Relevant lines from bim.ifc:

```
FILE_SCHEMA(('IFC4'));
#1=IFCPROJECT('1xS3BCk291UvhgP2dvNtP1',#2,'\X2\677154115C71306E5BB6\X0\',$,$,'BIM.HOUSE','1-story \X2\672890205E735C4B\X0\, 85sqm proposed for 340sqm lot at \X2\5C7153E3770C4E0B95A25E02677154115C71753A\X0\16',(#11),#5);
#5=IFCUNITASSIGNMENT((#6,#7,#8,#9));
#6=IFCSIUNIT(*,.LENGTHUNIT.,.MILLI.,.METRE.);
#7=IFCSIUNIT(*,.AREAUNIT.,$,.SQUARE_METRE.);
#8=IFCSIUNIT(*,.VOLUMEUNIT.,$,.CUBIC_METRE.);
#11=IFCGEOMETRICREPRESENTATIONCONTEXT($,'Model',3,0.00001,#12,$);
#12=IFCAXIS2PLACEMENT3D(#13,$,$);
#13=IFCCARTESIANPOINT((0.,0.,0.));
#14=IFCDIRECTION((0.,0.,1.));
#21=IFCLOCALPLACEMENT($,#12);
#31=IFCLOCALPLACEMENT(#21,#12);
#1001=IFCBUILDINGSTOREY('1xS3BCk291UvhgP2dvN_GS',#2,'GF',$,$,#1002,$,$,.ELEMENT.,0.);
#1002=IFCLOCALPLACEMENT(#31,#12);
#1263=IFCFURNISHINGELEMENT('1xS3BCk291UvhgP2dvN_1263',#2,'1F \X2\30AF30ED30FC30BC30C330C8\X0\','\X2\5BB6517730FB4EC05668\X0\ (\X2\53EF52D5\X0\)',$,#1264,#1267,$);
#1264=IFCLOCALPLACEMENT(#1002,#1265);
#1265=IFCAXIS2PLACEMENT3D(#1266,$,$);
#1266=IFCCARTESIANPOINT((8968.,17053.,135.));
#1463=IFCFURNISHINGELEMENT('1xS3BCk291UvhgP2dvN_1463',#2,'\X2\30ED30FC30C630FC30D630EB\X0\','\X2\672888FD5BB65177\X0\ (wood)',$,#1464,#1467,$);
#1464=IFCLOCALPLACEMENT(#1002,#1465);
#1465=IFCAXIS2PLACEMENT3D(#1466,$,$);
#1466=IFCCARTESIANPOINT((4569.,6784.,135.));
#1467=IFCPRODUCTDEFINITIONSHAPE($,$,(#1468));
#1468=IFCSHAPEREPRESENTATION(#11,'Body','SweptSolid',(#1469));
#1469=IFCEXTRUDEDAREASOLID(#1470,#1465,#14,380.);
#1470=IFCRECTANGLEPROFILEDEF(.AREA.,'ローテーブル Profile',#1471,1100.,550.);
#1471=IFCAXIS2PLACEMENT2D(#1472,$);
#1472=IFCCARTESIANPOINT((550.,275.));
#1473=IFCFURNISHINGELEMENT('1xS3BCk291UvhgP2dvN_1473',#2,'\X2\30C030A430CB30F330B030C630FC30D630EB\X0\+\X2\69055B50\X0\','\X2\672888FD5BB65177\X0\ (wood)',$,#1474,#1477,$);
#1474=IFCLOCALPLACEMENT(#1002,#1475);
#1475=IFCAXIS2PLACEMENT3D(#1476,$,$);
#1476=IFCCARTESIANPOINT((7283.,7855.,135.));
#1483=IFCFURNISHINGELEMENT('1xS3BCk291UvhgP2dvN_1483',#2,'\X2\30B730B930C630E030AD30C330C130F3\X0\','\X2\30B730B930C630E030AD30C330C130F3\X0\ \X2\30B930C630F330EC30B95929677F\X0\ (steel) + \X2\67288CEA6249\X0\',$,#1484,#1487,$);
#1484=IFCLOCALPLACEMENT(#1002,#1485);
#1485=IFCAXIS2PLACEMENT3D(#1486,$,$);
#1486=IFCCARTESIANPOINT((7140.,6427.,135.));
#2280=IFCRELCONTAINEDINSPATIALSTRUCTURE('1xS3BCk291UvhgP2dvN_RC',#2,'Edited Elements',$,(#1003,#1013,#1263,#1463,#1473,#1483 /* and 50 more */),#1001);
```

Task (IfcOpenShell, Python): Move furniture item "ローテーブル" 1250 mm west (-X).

```python
import ifcopenshell
import ifcopenshell.api.geometry
import ifcopenshell.util.placement
import ifcopenshell.util.unit

model = ifcopenshell.open("bim.ifc")
unit_scale = ifcopenshell.util.unit.calculate_unit_scale(model)

item = model.by_id(1463)
matrix = ifcopenshell.util.placement.get_local_placement(item.ObjectPlacement)
matrix[0, 3] -= 1.25 / unit_scale
ifcopenshell.api.geometry.edit_object_placement(model, product=item, matrix=matrix, is_si=False)

print(ifcopenshell.util.placement.get_local_placement(item.ObjectPlacement).round(3) + 0.0)

model.write("bim-out.ifc")
```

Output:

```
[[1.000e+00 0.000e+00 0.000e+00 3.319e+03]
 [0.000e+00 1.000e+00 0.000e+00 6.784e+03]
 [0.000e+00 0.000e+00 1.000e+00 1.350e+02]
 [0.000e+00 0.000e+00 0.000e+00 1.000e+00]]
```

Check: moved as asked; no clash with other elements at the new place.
